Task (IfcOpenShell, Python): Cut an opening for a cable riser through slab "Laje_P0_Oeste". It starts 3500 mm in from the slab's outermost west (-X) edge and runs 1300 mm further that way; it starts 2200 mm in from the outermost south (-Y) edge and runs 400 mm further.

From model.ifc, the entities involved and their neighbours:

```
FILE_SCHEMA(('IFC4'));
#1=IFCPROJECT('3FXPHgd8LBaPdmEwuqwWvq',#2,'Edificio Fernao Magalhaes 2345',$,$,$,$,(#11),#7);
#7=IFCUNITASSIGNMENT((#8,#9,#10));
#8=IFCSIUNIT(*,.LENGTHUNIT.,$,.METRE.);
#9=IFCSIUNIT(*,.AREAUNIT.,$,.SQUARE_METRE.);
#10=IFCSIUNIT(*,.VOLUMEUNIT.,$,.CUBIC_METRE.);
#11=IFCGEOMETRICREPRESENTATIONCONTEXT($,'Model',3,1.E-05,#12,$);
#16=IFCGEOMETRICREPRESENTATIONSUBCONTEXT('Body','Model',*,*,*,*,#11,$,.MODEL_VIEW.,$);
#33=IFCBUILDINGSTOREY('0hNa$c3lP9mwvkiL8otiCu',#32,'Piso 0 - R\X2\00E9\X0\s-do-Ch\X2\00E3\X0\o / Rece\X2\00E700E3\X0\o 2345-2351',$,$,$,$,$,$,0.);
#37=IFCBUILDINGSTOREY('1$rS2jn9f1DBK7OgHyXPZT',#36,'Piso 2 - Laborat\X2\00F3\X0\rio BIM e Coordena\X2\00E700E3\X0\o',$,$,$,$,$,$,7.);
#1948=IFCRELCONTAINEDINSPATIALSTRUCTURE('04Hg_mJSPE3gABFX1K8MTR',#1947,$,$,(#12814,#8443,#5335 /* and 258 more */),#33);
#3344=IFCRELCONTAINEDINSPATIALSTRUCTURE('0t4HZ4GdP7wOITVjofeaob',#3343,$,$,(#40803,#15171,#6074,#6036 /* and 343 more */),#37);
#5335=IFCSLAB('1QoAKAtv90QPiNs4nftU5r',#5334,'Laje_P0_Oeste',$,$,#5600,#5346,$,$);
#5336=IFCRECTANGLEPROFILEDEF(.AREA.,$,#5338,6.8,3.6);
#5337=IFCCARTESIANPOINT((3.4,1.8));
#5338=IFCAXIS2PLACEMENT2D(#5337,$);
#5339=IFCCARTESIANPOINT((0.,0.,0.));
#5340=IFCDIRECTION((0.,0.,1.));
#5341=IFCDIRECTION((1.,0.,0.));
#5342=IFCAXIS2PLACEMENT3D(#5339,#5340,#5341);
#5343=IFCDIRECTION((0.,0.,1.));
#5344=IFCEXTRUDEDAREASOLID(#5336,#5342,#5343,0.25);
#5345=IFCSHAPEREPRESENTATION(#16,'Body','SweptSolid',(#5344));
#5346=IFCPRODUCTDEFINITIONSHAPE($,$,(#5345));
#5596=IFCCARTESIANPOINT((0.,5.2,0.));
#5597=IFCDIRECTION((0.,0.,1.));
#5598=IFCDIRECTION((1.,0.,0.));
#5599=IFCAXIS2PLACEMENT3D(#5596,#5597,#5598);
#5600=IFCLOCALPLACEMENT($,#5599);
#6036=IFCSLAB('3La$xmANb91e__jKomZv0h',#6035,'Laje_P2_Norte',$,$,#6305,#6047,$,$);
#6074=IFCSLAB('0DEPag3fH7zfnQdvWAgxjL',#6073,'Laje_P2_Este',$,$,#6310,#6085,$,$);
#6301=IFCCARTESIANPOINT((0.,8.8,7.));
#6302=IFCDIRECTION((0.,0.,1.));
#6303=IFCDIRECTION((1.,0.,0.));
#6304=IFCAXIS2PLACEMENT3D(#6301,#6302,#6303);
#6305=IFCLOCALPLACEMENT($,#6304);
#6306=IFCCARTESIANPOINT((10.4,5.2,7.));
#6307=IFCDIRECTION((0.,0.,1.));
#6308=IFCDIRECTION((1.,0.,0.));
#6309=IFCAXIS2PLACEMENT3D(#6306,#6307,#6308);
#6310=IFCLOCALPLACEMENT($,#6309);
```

```python
import numpy as np
import ifcopenshell
import ifcopenshell.api.feature
import ifcopenshell.api.geometry
import ifcopenshell.api.root
import ifcopenshell.geom
import ifcopenshell.util.placement
import ifcopenshell.util.representation
import ifcopenshell.util.shape
import ifcopenshell.util.unit

model = ifcopenshell.open("model.ifc")
unit_scale = ifcopenshell.util.unit.calculate_unit_scale(model)
settings = ifcopenshell.geom.settings()


def volume(element):
    """Net volume in cubic metres, openings subtracted."""
    shape = ifcopenshell.geom.create_shape(settings, element)
    return ifcopenshell.util.shape.get_volume(shape.geometry)


slab = model.by_guid("1QoAKAtv90QPiNs4nftU5r")
before = volume(slab)

# Extent in the slab's own axes, in metres. The edges named are its -X and -Y sides.
slab_shape = ifcopenshell.geom.create_shape(settings, slab)
vertices = ifcopenshell.util.shape.get_vertices(slab_shape.geometry)
x_min, y_min, bottom = vertices.min(axis=0)
top = vertices[:, 2].max()

opening = ifcopenshell.api.root.create_entity(model, ifc_class="IfcOpeningElement", name="Cable riser opening", predefined_type="OPENING")
context = ifcopenshell.util.representation.get_context(model, "Model", "Body", "MODEL_VIEW")
width, depth = 1.3, 0.4
outline = [(0.0, 0.0), (width, 0.0), (width, depth), (0.0, depth), (0.0, 0.0)]
# Overshoot both faces by 50 mm so the cut is clean.
shape = ifcopenshell.api.geometry.add_slab_representation(
    model, context=context, depth=top - bottom + 0.1, polyline=outline
)
ifcopenshell.api.geometry.assign_representation(model, product=opening, representation=shape)

matrix = ifcopenshell.util.placement.get_local_placement(slab.ObjectPlacement)
matrix[:, 3] = matrix @ np.append(np.array([x_min + 3.5, y_min + 2.2, bottom - 0.05]) / unit_scale, 1.0)
ifcopenshell.api.geometry.edit_object_placement(model, product=opening, matrix=matrix, is_si=False)
ifcopenshell.api.feature.add_feature(model, feature=opening, element=slab)

after = volume(slab)

print(f"slab volume {before:.3f} -> {after:.3f} m3")

model.write("model_edited.ifc")
```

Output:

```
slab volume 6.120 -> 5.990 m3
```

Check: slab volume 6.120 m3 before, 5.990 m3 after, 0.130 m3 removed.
